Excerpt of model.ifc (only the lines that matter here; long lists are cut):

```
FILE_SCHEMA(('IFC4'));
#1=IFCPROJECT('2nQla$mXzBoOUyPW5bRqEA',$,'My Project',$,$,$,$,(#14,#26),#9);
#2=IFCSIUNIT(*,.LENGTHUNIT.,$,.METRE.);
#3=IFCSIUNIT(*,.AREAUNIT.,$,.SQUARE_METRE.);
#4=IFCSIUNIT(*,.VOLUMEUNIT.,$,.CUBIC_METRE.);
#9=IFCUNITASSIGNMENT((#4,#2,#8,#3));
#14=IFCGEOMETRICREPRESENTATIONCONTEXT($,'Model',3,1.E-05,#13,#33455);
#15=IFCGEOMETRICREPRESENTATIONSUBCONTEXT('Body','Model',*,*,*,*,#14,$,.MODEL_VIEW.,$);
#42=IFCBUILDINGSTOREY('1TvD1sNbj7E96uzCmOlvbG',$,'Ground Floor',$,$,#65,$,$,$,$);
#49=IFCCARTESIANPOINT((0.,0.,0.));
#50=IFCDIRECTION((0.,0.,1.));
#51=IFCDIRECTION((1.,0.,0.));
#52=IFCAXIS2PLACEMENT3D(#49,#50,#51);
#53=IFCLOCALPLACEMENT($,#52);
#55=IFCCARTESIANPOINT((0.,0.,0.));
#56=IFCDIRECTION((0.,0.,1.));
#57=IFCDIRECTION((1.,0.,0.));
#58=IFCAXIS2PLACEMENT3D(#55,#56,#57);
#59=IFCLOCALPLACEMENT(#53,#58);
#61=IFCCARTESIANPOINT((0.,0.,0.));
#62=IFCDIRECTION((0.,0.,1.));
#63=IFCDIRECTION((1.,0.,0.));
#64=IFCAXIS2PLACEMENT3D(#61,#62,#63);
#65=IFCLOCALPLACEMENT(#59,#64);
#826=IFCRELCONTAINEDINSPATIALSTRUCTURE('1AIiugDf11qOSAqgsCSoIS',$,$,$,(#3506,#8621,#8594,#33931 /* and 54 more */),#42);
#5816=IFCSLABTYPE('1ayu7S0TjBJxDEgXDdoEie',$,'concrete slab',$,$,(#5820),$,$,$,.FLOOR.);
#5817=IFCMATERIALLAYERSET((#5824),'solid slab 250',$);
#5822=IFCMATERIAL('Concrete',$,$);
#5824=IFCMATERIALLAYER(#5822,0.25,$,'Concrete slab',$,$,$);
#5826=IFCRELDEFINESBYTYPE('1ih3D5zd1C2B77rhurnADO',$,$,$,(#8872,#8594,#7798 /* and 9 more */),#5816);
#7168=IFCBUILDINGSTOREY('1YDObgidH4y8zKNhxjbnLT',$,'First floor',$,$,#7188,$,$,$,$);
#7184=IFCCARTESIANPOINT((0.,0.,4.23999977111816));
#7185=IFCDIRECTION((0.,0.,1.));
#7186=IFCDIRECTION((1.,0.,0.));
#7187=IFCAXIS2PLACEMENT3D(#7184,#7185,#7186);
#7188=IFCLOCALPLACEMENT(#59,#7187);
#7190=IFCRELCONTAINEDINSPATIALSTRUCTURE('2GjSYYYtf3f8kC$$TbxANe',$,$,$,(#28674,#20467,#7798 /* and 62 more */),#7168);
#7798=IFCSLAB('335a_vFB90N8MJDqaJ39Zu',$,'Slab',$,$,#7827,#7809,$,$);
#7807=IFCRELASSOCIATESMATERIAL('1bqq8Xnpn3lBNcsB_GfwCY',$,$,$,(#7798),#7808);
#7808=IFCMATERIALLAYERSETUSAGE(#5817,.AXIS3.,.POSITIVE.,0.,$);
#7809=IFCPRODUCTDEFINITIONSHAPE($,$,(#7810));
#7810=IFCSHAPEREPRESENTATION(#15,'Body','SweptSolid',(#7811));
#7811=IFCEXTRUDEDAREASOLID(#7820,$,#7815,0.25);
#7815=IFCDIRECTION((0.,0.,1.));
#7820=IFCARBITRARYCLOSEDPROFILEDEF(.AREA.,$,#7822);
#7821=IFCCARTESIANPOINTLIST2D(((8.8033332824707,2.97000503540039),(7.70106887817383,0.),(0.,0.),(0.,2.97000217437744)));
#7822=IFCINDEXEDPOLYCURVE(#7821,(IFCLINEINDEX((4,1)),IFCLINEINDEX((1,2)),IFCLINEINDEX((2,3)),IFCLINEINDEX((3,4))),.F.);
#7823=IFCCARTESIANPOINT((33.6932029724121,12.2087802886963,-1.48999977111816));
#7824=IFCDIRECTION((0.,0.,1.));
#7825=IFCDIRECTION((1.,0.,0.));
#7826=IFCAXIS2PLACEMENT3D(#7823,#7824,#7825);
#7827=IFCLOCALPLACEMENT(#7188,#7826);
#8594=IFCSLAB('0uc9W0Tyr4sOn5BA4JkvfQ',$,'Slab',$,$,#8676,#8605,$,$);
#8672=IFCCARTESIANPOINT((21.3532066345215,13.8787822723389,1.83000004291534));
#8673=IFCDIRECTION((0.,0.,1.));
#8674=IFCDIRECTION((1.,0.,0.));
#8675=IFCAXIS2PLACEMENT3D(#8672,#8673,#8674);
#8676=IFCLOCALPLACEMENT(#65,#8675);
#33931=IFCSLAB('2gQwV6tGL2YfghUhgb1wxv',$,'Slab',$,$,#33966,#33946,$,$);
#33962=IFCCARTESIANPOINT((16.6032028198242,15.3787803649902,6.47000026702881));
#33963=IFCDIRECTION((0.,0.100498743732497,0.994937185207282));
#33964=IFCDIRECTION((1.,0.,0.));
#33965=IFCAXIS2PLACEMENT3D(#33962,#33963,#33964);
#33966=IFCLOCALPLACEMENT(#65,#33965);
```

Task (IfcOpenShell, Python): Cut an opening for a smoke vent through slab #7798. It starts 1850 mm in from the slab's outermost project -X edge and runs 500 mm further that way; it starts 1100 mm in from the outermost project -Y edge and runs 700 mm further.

```python
import numpy as np
import ifcopenshell
import ifcopenshell.api.feature
import ifcopenshell.api.geometry
import ifcopenshell.api.root
import ifcopenshell.geom
import ifcopenshell.util.placement
import ifcopenshell.util.representation
import ifcopenshell.util.shape
import ifcopenshell.util.unit

model = ifcopenshell.open("model.ifc")
unit_scale = ifcopenshell.util.unit.calculate_unit_scale(model)
settings = ifcopenshell.geom.settings()


def volume(element):
    """Net volume in cubic metres, openings subtracted."""
    shape = ifcopenshell.geom.create_shape(settings, element)
    return ifcopenshell.util.shape.get_volume(shape.geometry)


slab = model.by_id(7798)
before = volume(slab)

# Extent in the slab's own axes, in metres. The edges named are its -X and -Y sides.
slab_shape = ifcopenshell.geom.create_shape(settings, slab)
vertices = ifcopenshell.util.shape.get_vertices(slab_shape.geometry)
x_min, y_min, bottom = vertices.min(axis=0)
top = vertices[:, 2].max()

opening = ifcopenshell.api.root.create_entity(model, ifc_class="IfcOpeningElement", name="Smoke vent opening", predefined_type="OPENING")
context = ifcopenshell.util.representation.get_context(model, "Model", "Body", "MODEL_VIEW")
width, depth = 0.5, 0.7
outline = [(0.0, 0.0), (width, 0.0), (width, depth), (0.0, depth), (0.0, 0.0)]
# Overshoot both faces by 50 mm so the cut is clean.
shape = ifcopenshell.api.geometry.add_slab_representation(
    model, context=context, depth=top - bottom + 0.1, polyline=outline
)
ifcopenshell.api.geometry.assign_representation(model, product=opening, representation=shape)

matrix = ifcopenshell.util.placement.get_local_placement(slab.ObjectPlacement)
matrix[:, 3] = matrix @ np.append(np.array([x_min + 1.85, y_min + 1.1, bottom - 0.05]) / unit_scale, 1.0)
ifcopenshell.api.geometry.edit_object_placement(model, product=opening, matrix=matrix, is_si=False)
ifcopenshell.api.feature.add_feature(model, feature=opening, element=slab)

after = volume(slab)

print(f"slab volume {before:.3f} -> {after:.3f} m3")

model.write("model_rev.ifc")
```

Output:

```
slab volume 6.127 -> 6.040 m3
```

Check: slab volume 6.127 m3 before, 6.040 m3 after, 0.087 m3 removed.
